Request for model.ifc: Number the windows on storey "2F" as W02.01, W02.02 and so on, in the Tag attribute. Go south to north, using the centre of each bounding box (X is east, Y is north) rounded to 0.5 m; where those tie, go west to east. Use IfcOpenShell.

First a look at what the model holds.

```python
import ifcopenshell
import ifcopenshell.util.element
import ifcopenshell.util.placement

model = ifcopenshell.open("model.ifc")
print(model.schema)
storey = next(s for s in model.by_type("IfcBuildingStorey") if s.Name == "2F")
windows = [e for e in ifcopenshell.util.element.get_decomposition(storey) if e.is_a("IfcWindow")]
for e in sorted(windows, key=lambda e: e.id()):
    origin = ifcopenshell.util.placement.get_local_placement(e.ObjectPlacement)[:3, 3]
    print(e.id(), e.Tag, e.Name, origin.round(2) + 0.0, sep=" | ")
```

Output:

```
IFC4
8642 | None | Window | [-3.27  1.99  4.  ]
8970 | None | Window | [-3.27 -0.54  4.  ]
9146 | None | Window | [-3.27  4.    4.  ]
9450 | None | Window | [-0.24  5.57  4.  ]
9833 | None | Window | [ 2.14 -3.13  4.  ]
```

```python
import ifcopenshell
import ifcopenshell.geom
import ifcopenshell.util.element
import ifcopenshell.util.shape

model = ifcopenshell.open("model.ifc")
settings = ifcopenshell.geom.settings()
settings.set("use-world-coords", True)


def centre(element):
    shape = ifcopenshell.geom.create_shape(settings, element)
    return ifcopenshell.util.shape.get_bbox_centroid(shape.geometry)


storey = next(s for s in model.by_type("IfcBuildingStorey") if s.Name == "2F")
windows = [e for e in ifcopenshell.util.element.get_decomposition(storey) if e.is_a("IfcWindow")]

# Insertion points can sit at a corner or the storey origin, so sort by the geometry (in metres).
centres = {e: centre(e) for e in windows}
windows.sort(key=lambda e: (round(centres[e][1] / 0.5), centres[e][0]))

for i, e in enumerate(windows, start=1):
    number = f"W02.{i:02d}"
    e.Tag = number
    print(e.id(), number)

model.write("model_rev.ifc")
```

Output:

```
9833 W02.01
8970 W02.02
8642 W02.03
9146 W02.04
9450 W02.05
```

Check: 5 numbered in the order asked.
